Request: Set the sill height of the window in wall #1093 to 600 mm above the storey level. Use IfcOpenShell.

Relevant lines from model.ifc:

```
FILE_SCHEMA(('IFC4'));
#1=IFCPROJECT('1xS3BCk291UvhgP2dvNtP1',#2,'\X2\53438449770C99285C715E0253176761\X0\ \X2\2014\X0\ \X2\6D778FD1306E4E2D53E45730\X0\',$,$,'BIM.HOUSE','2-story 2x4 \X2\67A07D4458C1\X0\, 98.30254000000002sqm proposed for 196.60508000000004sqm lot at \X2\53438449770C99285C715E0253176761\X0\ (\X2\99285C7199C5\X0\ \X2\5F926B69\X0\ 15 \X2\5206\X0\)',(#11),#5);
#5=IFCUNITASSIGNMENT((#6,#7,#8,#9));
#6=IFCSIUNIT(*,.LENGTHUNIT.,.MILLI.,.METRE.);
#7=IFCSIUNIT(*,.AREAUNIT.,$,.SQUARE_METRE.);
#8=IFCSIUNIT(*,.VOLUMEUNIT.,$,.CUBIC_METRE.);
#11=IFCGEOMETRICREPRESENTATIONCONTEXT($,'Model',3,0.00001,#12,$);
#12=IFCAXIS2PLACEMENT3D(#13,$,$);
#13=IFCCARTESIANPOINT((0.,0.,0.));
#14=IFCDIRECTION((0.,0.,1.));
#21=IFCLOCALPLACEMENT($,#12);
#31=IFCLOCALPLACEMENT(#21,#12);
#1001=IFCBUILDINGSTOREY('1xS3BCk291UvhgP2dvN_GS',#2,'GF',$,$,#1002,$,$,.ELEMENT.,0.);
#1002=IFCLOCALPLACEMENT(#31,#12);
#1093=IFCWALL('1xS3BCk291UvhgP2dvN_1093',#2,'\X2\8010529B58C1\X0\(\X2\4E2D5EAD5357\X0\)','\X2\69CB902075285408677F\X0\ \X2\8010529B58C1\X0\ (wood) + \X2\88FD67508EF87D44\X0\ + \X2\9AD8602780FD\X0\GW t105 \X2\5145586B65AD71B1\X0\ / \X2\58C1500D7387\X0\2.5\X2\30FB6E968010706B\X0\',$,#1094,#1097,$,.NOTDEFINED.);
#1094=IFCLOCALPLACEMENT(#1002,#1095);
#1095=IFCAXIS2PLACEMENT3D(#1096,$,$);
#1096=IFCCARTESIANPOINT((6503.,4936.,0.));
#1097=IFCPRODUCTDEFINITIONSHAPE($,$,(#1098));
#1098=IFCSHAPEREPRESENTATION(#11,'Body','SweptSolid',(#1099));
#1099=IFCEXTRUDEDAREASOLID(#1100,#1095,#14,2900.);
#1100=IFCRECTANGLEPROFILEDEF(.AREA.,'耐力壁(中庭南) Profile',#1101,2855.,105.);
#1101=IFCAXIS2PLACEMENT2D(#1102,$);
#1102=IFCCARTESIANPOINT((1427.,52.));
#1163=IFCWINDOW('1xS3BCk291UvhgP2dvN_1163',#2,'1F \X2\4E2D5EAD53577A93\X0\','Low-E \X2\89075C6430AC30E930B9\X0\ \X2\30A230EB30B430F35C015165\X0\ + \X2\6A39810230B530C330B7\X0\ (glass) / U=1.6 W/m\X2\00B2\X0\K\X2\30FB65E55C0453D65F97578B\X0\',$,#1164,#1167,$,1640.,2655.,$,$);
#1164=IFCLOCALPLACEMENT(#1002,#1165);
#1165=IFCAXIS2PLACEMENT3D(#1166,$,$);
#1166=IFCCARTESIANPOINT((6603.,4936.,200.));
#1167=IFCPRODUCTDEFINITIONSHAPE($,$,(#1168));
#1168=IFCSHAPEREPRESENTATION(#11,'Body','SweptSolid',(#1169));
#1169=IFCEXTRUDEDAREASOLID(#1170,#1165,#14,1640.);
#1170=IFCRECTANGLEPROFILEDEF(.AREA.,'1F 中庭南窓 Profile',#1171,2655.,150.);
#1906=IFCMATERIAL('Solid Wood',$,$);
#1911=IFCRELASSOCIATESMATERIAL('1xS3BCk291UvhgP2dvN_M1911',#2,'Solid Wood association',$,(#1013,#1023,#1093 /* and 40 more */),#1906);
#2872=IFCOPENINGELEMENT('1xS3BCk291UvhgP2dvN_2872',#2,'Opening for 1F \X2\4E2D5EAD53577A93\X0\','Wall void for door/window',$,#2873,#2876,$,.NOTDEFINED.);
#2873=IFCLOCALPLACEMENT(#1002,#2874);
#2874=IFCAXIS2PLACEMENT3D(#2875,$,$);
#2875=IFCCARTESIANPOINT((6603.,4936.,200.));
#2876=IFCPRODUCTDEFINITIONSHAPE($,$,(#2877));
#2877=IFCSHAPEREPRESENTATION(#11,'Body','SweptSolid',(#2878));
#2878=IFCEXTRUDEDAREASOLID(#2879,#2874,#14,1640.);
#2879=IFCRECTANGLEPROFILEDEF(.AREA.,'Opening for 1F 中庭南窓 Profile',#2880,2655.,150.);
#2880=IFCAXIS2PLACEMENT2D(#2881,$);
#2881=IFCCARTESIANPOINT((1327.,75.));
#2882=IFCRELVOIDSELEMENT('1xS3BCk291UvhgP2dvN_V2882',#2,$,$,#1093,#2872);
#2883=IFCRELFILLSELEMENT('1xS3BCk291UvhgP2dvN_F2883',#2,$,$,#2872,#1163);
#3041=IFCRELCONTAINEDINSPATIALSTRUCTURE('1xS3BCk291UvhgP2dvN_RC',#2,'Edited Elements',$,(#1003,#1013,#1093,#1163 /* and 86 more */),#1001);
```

```python
import numpy as np
import ifcopenshell
import ifcopenshell.api.geometry
import ifcopenshell.geom
import ifcopenshell.util.element
import ifcopenshell.util.placement
import ifcopenshell.util.shape
import ifcopenshell.util.unit

model = ifcopenshell.open("model.ifc")
unit_scale = ifcopenshell.util.unit.calculate_unit_scale(model)

window = model.by_guid("1xS3BCk291UvhgP2dvN_1163")
opening = window.FillsVoids[0].RelatingOpeningElement
storey = ifcopenshell.util.element.get_container(window, ifc_class="IfcBuildingStorey")
level = ifcopenshell.util.placement.get_local_placement(storey.ObjectPlacement)[2, 3]

# The opening's origin need not be at the sill, so measure its lowest point.
shape = ifcopenshell.geom.create_shape(ifcopenshell.geom.settings(), opening)
bottom = ifcopenshell.util.shape.get_shape_bottom_elevation(shape, shape.geometry) / unit_scale
dz = level + 0.6 / unit_scale - bottom

shift = np.array([0.0, 0.0, dz])
# The window is not placed relative to its opening, so move both.
for product in (opening, window):
    matrix = ifcopenshell.util.placement.get_local_placement(product.ObjectPlacement)
    matrix[:3, 3] += shift
    ifcopenshell.api.geometry.edit_object_placement(model, product=product, matrix=matrix, is_si=False)

print(f"moved by {dz * unit_scale:+.3f} m")

model.write("model_rev.ifc")
```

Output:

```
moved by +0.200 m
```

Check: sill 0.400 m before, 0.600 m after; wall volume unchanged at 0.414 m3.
